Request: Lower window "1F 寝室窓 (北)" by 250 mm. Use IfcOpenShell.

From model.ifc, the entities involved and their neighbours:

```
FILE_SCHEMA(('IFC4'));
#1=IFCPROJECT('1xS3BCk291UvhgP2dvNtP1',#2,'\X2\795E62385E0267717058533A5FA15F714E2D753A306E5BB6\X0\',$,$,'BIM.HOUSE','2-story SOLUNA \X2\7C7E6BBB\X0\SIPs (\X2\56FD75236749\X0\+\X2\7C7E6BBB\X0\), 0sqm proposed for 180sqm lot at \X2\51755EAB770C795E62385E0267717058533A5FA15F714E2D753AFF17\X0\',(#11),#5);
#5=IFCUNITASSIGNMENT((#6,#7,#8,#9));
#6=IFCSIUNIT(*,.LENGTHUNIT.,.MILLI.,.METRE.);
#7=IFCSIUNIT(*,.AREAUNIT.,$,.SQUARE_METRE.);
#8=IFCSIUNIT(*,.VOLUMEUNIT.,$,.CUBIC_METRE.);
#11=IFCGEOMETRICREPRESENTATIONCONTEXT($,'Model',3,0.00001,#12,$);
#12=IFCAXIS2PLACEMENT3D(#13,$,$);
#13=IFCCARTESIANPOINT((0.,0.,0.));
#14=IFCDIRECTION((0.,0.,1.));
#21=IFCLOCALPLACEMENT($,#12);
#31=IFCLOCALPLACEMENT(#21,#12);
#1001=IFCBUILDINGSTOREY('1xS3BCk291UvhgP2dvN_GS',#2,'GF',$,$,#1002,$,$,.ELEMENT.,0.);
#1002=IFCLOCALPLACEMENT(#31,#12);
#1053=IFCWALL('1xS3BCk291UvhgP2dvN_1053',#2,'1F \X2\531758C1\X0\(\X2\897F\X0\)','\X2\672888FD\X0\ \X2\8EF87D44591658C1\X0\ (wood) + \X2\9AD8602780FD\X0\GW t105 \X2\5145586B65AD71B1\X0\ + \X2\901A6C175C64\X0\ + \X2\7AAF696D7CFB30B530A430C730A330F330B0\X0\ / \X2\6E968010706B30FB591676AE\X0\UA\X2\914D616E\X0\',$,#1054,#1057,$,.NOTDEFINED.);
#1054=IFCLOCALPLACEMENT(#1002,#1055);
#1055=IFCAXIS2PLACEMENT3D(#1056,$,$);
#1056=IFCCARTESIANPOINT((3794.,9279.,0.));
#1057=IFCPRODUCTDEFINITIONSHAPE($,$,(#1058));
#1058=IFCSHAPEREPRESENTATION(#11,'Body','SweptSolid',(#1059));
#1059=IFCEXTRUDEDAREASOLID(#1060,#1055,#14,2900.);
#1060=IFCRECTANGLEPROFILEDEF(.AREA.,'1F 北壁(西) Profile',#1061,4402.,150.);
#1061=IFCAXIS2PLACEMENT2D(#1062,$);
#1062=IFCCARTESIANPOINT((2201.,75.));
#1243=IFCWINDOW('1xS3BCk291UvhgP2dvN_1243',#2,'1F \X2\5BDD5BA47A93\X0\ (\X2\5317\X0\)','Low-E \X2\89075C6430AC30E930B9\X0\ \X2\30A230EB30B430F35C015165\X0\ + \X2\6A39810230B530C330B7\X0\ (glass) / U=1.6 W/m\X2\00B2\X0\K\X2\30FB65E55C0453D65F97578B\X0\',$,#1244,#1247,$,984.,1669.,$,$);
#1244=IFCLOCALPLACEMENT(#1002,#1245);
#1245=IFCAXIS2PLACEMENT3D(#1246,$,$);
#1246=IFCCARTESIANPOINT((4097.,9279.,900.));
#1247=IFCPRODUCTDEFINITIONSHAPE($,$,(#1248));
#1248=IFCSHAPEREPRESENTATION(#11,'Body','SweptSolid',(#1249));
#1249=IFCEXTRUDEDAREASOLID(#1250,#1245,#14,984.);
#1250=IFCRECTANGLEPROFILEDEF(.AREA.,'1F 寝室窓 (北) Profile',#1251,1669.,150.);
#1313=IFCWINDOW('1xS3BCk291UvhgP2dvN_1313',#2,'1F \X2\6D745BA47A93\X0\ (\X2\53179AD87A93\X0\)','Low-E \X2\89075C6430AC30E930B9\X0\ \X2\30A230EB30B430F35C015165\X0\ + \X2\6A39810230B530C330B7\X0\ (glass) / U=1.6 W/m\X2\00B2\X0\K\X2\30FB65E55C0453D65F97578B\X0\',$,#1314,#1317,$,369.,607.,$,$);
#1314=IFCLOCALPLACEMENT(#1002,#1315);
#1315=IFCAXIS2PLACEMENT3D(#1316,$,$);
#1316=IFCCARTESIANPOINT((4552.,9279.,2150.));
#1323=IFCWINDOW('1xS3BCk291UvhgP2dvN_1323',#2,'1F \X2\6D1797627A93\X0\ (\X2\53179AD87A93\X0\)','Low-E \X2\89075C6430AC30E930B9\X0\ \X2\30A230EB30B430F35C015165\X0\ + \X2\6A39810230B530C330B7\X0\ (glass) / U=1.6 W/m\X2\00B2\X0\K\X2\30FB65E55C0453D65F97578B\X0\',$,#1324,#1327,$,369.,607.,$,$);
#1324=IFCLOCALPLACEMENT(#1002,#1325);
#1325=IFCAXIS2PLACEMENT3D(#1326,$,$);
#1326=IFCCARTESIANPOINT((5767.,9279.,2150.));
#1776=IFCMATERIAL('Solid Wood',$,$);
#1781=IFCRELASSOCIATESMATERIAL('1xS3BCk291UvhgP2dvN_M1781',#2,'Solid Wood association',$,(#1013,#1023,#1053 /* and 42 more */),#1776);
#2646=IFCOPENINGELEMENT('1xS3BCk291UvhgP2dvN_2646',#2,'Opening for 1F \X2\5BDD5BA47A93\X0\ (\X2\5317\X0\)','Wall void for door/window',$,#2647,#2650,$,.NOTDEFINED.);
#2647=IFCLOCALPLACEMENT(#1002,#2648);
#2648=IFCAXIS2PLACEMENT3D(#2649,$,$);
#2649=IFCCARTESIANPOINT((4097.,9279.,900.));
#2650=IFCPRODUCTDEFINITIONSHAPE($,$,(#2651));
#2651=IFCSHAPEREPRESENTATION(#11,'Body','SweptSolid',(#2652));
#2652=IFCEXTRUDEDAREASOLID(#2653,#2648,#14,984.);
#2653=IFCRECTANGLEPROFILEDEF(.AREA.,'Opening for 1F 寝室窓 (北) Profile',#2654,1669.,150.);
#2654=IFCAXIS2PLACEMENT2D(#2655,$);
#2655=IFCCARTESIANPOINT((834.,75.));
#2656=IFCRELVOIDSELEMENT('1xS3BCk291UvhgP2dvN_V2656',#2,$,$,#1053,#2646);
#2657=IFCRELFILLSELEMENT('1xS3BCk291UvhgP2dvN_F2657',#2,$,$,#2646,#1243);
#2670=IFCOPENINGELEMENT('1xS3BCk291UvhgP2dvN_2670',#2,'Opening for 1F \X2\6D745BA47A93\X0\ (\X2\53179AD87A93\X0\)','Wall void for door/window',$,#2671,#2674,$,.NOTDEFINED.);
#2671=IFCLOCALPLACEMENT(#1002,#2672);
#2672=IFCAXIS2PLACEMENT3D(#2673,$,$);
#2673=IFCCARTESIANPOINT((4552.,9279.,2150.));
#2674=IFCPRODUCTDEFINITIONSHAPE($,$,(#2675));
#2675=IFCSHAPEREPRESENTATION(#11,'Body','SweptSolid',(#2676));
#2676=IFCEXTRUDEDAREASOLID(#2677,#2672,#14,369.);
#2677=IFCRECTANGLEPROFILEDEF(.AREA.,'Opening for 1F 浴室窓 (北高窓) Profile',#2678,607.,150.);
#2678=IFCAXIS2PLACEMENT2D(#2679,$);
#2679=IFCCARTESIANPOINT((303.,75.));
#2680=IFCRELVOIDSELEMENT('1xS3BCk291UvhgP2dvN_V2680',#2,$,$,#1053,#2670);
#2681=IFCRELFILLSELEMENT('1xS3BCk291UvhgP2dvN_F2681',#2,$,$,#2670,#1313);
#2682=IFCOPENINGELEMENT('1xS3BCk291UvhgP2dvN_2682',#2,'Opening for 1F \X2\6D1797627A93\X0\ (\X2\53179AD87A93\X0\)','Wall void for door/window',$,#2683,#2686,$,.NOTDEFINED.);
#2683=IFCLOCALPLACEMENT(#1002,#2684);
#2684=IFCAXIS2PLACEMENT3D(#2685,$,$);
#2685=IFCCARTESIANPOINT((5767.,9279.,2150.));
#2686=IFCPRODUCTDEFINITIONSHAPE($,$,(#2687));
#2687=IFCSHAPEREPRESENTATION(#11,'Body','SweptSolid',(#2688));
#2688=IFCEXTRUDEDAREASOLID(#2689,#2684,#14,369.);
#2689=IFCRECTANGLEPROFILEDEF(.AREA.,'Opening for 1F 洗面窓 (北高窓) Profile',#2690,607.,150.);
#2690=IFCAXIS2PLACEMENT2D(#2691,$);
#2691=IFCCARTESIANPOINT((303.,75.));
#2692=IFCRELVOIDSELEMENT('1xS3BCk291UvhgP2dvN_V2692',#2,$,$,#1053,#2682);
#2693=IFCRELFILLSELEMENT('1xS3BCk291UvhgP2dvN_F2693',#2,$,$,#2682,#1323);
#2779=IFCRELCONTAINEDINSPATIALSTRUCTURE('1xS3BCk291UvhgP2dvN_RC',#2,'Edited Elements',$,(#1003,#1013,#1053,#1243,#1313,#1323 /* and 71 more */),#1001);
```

```python
import numpy as np
import ifcopenshell
import ifcopenshell.api.geometry
import ifcopenshell.util.placement
import ifcopenshell.util.unit

model = ifcopenshell.open("model.ifc")
unit_scale = ifcopenshell.util.unit.calculate_unit_scale(model)

window = model.by_id(1243)
opening = window.FillsVoids[0].RelatingOpeningElement
dz = -0.25 / unit_scale

shift = np.array([0.0, 0.0, dz])
# The window is not placed relative to its opening, so move both.
for product in (opening, window):
    matrix = ifcopenshell.util.placement.get_local_placement(product.ObjectPlacement)
    matrix[:3, 3] += shift
    ifcopenshell.api.geometry.edit_object_placement(model, product=product, matrix=matrix, is_si=False)

print(f"moved by {dz * unit_scale:+.3f} m")

model.write("model_v2.ifc")
```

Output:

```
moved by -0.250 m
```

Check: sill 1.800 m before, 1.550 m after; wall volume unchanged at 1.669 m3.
